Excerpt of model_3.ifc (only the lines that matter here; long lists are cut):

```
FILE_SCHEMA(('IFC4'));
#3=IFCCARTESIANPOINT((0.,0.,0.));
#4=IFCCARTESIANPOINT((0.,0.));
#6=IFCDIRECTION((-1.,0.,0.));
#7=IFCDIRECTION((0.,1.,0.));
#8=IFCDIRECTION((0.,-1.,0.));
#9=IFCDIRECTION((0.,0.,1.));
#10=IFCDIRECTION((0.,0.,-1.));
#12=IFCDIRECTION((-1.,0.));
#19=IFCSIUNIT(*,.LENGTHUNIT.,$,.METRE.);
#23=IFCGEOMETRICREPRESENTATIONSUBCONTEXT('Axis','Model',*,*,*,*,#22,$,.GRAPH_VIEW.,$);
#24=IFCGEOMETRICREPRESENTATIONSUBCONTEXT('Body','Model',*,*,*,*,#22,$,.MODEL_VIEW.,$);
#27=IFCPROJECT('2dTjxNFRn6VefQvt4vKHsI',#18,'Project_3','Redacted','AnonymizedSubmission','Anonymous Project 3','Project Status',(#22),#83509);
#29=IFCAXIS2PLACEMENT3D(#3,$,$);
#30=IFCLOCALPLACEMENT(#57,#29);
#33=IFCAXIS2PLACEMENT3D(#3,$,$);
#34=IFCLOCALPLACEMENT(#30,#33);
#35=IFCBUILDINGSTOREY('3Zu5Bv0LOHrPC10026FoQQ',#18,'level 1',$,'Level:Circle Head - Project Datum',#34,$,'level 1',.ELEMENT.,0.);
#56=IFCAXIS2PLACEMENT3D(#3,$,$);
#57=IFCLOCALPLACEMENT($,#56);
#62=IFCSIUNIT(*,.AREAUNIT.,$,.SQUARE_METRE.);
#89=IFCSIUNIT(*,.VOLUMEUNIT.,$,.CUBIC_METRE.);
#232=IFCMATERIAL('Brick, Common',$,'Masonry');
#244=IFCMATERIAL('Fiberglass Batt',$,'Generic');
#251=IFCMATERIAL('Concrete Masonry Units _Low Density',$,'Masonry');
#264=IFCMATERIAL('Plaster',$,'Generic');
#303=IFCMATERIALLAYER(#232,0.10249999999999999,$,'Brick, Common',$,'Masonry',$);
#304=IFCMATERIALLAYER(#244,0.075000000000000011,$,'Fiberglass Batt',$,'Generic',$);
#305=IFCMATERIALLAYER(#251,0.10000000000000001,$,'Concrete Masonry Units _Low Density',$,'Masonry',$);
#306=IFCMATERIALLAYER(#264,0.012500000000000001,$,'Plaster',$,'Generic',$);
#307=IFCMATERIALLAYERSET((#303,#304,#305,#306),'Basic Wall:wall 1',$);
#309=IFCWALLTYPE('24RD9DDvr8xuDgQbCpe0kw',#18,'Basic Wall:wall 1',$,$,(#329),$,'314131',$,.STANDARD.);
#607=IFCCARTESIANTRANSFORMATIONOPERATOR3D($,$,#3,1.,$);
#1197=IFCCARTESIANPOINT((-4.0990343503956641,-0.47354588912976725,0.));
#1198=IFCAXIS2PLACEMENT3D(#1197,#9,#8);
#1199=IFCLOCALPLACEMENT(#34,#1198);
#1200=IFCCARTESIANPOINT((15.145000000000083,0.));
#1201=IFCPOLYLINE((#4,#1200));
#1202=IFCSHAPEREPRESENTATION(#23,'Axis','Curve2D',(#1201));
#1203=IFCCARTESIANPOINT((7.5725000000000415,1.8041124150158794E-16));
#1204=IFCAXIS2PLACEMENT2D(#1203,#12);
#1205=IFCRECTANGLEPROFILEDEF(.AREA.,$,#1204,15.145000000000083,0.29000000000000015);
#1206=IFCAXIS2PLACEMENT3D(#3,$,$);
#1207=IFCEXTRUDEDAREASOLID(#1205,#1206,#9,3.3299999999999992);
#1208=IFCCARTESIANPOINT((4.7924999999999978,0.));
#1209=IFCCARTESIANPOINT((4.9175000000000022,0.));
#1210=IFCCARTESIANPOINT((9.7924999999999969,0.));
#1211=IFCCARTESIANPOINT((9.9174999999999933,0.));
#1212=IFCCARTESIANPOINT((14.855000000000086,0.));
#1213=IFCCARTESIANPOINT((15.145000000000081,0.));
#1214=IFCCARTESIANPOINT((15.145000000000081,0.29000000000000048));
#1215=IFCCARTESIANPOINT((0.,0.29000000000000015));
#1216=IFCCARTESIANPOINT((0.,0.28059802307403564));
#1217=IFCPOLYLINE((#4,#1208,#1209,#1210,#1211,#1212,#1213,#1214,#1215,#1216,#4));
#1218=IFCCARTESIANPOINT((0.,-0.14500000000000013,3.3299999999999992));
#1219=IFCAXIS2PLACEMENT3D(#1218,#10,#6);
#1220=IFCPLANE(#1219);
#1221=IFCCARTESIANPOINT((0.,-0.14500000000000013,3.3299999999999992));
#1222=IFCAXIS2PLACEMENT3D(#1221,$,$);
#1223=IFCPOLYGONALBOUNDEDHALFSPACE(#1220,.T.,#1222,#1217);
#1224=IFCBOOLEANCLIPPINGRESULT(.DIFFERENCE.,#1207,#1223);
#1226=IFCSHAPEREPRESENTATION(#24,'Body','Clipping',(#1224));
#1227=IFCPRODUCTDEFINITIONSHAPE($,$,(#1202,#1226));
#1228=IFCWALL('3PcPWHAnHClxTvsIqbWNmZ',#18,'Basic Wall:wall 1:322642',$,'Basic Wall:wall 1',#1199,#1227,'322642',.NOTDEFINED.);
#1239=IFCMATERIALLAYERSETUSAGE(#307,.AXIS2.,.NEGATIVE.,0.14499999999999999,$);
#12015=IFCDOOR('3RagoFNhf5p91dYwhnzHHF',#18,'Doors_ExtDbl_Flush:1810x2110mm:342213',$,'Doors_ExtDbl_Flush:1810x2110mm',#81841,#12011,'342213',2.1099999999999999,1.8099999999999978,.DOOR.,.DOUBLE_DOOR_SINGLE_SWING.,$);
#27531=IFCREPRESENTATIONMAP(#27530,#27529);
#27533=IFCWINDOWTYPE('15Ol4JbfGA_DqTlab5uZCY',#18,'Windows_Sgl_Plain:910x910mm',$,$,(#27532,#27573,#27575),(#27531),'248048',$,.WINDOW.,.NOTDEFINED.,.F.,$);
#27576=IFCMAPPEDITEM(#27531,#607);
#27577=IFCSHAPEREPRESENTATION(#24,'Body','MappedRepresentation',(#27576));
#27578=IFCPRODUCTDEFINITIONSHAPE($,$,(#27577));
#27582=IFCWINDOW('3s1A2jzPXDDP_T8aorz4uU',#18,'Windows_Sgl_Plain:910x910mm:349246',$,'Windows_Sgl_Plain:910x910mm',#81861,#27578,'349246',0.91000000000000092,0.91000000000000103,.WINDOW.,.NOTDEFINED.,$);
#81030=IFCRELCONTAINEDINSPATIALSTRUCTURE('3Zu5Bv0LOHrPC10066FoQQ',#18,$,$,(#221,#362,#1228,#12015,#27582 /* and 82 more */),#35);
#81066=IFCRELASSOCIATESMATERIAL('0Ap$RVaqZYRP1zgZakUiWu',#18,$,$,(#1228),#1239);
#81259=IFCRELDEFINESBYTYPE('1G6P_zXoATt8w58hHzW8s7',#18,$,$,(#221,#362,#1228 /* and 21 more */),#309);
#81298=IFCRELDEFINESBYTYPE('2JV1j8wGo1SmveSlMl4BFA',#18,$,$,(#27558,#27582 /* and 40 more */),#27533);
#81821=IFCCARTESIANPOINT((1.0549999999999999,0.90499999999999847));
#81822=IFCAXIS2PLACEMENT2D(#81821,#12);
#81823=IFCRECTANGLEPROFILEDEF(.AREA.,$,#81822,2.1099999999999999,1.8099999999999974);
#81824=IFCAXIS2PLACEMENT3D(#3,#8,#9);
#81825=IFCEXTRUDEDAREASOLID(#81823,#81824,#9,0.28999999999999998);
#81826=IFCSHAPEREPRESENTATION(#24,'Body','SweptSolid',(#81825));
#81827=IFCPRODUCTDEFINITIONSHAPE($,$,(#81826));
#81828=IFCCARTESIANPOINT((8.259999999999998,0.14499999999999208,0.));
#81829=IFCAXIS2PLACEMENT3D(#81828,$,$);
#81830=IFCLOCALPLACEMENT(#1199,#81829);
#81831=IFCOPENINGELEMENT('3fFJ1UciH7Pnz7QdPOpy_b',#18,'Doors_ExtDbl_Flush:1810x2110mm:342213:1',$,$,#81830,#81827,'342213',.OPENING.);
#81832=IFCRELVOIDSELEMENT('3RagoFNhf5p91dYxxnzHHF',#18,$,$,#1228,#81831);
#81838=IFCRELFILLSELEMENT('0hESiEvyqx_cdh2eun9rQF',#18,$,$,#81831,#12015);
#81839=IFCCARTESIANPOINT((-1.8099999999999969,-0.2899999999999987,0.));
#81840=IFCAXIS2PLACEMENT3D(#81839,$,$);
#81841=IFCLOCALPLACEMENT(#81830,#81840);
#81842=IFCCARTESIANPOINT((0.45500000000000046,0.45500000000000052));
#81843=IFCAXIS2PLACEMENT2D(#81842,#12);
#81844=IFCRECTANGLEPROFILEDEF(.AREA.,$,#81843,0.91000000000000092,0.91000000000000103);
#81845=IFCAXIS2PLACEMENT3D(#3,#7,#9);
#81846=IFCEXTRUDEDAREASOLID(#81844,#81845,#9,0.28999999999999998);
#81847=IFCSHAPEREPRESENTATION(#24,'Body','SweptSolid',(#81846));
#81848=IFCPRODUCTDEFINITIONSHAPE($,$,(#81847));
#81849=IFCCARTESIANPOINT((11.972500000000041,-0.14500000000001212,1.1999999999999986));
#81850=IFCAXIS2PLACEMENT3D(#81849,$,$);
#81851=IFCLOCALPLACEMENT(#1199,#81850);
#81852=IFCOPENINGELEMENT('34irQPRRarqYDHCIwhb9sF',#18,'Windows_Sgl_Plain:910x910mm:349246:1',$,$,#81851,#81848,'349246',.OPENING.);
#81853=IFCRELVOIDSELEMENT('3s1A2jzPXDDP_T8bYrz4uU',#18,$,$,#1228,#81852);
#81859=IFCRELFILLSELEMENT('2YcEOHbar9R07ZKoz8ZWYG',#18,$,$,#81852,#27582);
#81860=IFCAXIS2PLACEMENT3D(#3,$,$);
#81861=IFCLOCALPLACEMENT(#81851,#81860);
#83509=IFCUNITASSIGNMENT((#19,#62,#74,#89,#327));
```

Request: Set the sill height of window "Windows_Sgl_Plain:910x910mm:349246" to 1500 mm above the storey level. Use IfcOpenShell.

```python
import numpy as np
import ifcopenshell
import ifcopenshell.api.geometry
import ifcopenshell.geom
import ifcopenshell.util.element
import ifcopenshell.util.placement
import ifcopenshell.util.shape
import ifcopenshell.util.unit

model = ifcopenshell.open("model_3.ifc")
unit_scale = ifcopenshell.util.unit.calculate_unit_scale(model)

window = model.by_guid("3s1A2jzPXDDP_T8aorz4uU")
opening = window.FillsVoids[0].RelatingOpeningElement
storey = ifcopenshell.util.element.get_container(window, ifc_class="IfcBuildingStorey")
level = ifcopenshell.util.placement.get_local_placement(storey.ObjectPlacement)[2, 3]

# The opening's origin need not be at the sill, so measure its lowest point.
shape = ifcopenshell.geom.create_shape(ifcopenshell.geom.settings(), opening)
bottom = ifcopenshell.util.shape.get_shape_bottom_elevation(shape, shape.geometry) / unit_scale
dz = level + 1.5 - bottom

shift = np.array([0.0, 0.0, dz])
# The window is placed relative to its opening, so it follows when the opening moves.
matrix = ifcopenshell.util.placement.get_local_placement(opening.ObjectPlacement)
matrix[:3, 3] += shift
ifcopenshell.api.geometry.edit_object_placement(
    model, product=opening, matrix=matrix, is_si=False, should_transform_children=True
)

print(f"moved by {dz * unit_scale:+.3f} m")

model.write("model_3_rev.ifc")
```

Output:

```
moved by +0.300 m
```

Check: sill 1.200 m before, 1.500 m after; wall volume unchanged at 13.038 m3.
